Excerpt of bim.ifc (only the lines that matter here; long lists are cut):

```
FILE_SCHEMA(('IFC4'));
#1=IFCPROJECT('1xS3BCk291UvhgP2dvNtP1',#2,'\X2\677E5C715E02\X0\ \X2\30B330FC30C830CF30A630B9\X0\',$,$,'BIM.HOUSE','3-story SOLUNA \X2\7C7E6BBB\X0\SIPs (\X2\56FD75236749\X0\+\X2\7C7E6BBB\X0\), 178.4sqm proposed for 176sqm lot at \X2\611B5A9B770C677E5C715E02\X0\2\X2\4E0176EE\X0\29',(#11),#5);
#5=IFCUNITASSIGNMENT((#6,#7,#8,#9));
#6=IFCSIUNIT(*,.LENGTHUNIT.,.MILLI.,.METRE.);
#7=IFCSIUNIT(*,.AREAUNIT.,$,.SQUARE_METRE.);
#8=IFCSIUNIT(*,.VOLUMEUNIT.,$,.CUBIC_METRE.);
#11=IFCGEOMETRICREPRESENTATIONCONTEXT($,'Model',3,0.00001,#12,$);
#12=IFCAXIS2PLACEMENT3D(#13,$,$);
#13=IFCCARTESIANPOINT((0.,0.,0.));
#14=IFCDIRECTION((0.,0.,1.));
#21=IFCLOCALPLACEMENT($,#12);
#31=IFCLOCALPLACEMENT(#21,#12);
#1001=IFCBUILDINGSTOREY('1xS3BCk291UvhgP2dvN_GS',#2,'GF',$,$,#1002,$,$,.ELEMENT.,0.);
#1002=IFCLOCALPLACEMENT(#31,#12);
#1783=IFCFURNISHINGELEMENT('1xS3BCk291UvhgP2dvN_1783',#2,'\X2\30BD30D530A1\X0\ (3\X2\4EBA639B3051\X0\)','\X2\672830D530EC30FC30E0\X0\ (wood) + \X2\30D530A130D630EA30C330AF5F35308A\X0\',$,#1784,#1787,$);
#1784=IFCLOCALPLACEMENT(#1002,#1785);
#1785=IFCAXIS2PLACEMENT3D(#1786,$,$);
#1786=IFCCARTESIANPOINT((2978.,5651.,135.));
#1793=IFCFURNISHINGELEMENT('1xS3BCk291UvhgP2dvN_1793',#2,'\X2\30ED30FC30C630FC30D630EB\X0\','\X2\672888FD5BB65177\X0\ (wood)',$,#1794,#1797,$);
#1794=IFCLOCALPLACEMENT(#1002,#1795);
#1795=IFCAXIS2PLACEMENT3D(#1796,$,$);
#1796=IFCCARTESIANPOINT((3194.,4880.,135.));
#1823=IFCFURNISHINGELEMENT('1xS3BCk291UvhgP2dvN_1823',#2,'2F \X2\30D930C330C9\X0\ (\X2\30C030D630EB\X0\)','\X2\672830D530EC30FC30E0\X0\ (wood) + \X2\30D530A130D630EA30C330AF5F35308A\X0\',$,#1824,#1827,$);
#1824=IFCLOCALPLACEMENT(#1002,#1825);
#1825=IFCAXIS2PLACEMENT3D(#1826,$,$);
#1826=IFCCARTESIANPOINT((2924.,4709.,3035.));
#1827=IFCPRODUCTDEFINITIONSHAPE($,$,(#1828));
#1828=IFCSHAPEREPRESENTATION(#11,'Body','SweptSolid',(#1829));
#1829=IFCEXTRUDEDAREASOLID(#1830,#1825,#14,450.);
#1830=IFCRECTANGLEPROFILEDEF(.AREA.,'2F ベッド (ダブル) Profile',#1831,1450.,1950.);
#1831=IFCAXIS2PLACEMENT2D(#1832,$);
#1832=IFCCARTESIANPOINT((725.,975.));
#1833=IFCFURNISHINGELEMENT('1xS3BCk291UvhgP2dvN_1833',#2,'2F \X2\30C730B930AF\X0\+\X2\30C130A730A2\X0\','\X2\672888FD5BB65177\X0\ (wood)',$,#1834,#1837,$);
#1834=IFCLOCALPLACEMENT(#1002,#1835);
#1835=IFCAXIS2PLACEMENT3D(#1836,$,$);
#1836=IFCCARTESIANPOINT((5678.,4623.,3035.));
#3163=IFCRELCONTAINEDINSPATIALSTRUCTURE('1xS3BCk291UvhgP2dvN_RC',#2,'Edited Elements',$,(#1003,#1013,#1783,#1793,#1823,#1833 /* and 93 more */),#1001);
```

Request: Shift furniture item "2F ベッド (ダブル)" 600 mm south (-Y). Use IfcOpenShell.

```python
import ifcopenshell
import ifcopenshell.api.geometry
import ifcopenshell.util.placement

model = ifcopenshell.open("bim.ifc")

item = model.by_id(1823)
matrix = ifcopenshell.util.placement.get_local_placement(item.ObjectPlacement)
matrix[1, 3] -= 600.0
ifcopenshell.api.geometry.edit_object_placement(model, product=item, matrix=matrix, is_si=False)

print(ifcopenshell.util.placement.get_local_placement(item.ObjectPlacement).round(3) + 0.0)

model.write("bim_v2.ifc")
```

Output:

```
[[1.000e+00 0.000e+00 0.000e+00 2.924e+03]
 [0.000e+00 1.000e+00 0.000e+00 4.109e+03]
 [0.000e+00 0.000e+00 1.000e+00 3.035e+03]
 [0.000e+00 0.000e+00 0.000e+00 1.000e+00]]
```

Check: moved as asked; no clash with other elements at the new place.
